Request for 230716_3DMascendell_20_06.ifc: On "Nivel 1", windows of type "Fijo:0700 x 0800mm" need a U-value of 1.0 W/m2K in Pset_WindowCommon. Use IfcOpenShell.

First a look at what the model holds.

```python
import ifcopenshell
import ifcopenshell.util.element

model = ifcopenshell.open("230716_3DMascendell_20_06.ifc")
print(model.schema)
storey = next(s for s in model.by_type("IfcBuildingStorey") if s.Name == "Nivel 1")
windows = [e for e in ifcopenshell.util.element.get_decomposition(storey) if e.is_a("IfcWindow")]
seen = {}
for e in windows:
    element_type = ifcopenshell.util.element.get_type(e)
    key = (element_type.Name if element_type != e and element_type else None, ifcopenshell.util.element.get_pset(e, "Pset_WindowCommon", "ThermalTransmittance"))
    seen[key] = seen.get(key, 0) + 1
for (name, value), count in sorted(seen.items(), key=str):
    print(count, "x", name, "|", value)
```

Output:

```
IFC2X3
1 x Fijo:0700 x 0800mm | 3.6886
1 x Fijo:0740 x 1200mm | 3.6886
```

```python
import ifcopenshell
import ifcopenshell.api.pset
import ifcopenshell.util.element

model = ifcopenshell.open("230716_3DMascendell_20_06.ifc")

storey = next(s for s in model.by_type("IfcBuildingStorey") if s.Name == "Nivel 1")
windows = [e for e in ifcopenshell.util.element.get_decomposition(storey) if e.is_a("IfcWindow")]

count = 0
for e in windows:
    element_type = ifcopenshell.util.element.get_type(e)
    if element_type in (None, e) or element_type.Name != "Fijo:0700 x 0800mm":
        continue
    # add_pset returns the element's existing set when there is one.
    pset = ifcopenshell.api.pset.add_pset(model, product=e, name="Pset_WindowCommon")
    ifcopenshell.api.pset.edit_pset(model, pset=pset, properties={"ThermalTransmittance": 1.0})
    count += 1

print(count, "windows updated")

model.write("230716_3DMascendell_20_06-out.ifc")
```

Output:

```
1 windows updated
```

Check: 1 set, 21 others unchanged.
